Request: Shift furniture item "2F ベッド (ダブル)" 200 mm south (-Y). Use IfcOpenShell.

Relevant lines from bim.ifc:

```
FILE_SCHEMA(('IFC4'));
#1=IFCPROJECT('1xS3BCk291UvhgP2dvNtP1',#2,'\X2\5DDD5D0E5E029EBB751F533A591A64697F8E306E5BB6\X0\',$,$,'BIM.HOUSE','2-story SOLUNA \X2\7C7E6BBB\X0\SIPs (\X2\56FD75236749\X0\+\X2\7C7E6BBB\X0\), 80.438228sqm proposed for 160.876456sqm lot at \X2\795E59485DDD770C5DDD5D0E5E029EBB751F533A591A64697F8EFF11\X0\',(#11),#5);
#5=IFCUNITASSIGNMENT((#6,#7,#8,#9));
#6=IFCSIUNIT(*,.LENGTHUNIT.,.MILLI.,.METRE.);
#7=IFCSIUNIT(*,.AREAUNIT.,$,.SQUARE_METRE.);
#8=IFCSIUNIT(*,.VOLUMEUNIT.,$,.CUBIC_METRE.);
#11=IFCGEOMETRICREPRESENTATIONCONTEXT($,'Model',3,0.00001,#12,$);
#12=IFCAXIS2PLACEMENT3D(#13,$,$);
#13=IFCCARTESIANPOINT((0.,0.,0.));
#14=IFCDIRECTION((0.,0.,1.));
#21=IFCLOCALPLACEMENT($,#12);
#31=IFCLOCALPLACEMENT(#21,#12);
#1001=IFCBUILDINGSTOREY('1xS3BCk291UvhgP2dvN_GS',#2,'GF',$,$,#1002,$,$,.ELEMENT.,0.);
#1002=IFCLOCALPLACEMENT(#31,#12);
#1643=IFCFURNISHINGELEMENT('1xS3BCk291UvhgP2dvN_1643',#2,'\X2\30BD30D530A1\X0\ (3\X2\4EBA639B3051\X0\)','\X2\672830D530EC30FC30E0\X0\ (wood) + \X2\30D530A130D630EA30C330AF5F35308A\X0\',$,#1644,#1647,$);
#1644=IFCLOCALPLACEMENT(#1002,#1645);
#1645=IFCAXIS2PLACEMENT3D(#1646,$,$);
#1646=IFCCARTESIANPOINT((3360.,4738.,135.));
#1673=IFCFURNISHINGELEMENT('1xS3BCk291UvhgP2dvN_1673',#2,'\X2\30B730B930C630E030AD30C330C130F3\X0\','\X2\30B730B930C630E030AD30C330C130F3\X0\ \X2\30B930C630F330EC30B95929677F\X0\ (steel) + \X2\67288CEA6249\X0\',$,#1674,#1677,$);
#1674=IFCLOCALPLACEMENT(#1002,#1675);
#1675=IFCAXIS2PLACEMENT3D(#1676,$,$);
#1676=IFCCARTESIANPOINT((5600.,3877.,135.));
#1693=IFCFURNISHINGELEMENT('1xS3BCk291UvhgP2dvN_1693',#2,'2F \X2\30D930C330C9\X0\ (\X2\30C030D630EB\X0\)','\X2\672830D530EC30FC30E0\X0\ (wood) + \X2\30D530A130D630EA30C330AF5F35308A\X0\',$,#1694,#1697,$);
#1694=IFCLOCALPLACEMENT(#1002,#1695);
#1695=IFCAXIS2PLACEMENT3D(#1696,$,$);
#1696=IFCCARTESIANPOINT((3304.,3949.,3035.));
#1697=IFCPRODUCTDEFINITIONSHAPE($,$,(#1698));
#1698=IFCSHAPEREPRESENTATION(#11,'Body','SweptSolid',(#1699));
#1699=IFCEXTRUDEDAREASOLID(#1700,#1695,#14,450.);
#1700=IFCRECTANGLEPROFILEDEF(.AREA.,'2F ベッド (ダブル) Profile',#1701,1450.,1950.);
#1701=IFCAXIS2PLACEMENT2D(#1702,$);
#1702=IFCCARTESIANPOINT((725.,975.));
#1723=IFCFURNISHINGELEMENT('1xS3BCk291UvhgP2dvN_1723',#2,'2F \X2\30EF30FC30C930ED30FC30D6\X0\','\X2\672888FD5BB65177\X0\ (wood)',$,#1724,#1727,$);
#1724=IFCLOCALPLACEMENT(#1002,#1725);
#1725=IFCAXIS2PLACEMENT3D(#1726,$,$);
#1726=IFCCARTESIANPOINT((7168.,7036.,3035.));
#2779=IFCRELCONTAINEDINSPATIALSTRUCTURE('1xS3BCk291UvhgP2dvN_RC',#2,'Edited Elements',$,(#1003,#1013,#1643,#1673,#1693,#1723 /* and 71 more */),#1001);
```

```python
import ifcopenshell
import ifcopenshell.api.geometry
import ifcopenshell.util.placement

model = ifcopenshell.open("bim.ifc")

item = model.by_guid("1xS3BCk291UvhgP2dvN_1693")
matrix = ifcopenshell.util.placement.get_local_placement(item.ObjectPlacement)
matrix[1, 3] -= 200.0
ifcopenshell.api.geometry.edit_object_placement(model, product=item, matrix=matrix, is_si=False)

print(ifcopenshell.util.placement.get_local_placement(item.ObjectPlacement).round(3) + 0.0)

model.write("bim_updated.ifc")
```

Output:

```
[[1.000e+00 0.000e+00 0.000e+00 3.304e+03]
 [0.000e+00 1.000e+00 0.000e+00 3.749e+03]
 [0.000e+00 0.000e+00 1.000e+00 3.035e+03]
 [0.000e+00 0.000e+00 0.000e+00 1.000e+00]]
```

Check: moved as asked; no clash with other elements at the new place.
